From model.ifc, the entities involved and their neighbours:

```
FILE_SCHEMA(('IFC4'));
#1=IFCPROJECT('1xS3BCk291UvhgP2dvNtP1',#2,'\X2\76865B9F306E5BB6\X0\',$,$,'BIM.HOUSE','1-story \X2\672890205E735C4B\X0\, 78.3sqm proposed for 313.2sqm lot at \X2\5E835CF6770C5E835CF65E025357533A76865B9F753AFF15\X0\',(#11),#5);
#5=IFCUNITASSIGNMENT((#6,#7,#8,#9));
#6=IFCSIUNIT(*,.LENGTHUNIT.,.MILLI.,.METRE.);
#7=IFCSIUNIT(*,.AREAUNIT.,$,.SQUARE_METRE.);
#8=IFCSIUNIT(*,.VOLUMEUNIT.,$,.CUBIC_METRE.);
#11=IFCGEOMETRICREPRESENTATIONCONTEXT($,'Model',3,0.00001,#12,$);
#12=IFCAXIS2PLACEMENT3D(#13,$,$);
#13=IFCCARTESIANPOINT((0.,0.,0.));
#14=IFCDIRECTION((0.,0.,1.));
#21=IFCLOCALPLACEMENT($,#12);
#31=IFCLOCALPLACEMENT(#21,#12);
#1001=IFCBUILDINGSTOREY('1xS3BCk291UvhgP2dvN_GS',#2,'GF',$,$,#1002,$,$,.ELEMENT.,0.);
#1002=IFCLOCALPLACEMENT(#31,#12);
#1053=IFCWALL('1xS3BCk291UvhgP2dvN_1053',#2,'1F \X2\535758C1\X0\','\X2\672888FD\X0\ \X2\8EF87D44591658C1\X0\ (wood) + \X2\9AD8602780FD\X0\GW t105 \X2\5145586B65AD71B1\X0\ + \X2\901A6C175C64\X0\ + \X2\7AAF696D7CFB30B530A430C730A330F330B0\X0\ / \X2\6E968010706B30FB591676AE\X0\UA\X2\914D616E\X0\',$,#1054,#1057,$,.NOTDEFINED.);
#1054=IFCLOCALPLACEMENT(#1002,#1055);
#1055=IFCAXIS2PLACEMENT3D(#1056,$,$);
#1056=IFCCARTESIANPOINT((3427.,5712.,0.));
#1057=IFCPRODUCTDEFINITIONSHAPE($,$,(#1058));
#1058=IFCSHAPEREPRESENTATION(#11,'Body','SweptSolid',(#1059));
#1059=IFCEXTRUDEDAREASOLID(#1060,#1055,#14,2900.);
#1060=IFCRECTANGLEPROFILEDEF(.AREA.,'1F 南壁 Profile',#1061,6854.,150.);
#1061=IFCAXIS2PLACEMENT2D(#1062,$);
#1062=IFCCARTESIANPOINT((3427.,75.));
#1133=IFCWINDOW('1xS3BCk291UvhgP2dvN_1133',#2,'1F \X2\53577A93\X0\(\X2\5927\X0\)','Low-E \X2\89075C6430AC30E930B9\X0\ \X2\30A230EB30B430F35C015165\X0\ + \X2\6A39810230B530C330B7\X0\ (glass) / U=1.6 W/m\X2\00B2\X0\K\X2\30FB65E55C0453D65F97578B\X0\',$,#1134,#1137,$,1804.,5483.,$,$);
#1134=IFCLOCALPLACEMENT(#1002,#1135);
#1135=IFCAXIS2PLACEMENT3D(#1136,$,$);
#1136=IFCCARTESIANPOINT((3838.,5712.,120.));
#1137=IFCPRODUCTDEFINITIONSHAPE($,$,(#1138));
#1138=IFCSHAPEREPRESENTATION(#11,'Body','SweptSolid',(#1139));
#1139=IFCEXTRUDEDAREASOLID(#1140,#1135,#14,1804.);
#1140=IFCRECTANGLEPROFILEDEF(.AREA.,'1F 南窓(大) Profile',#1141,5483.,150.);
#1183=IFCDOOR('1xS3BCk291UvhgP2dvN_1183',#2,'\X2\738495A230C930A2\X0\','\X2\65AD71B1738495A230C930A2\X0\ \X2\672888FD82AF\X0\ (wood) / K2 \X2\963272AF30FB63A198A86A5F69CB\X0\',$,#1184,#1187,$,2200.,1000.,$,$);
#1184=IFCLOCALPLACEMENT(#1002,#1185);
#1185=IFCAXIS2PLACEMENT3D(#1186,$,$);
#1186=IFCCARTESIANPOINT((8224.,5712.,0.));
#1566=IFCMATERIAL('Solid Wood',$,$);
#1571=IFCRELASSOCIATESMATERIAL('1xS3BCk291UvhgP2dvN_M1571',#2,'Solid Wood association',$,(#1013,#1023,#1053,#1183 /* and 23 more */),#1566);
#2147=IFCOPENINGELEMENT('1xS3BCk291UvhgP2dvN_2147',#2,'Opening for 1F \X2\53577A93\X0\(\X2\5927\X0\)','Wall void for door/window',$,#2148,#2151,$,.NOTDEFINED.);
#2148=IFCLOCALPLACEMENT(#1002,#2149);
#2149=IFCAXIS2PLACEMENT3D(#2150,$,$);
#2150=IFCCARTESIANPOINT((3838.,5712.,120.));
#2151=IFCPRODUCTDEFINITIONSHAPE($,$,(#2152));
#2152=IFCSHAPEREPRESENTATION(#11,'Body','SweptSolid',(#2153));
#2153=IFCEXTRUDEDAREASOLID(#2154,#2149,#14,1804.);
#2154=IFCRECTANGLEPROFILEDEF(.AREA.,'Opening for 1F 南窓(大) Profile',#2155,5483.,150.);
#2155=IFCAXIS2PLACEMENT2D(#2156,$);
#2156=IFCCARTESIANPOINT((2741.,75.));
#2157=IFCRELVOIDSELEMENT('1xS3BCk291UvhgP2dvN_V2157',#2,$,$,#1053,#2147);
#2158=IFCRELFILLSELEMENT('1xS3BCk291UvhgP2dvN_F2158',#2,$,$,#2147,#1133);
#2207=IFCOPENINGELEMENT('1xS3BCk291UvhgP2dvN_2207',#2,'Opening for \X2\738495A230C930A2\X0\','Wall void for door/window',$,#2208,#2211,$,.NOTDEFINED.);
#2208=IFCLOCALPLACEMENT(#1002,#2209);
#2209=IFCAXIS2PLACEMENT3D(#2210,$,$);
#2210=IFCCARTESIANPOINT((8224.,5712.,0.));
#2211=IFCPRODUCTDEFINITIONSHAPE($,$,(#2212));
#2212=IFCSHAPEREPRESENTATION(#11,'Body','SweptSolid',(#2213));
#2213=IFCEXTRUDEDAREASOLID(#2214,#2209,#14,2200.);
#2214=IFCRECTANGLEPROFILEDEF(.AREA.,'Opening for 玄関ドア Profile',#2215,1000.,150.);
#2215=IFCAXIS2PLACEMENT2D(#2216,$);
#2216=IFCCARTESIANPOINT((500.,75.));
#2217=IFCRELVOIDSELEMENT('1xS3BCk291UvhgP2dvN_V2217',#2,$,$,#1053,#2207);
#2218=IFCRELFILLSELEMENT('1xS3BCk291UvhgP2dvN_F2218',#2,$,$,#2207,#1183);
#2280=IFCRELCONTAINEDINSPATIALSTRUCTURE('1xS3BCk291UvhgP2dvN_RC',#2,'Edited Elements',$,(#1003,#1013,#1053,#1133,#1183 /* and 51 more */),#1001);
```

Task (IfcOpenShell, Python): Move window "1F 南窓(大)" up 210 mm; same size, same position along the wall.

```python
import numpy as np
import ifcopenshell
import ifcopenshell.api.geometry
import ifcopenshell.util.placement
import ifcopenshell.util.unit

model = ifcopenshell.open("model.ifc")
unit_scale = ifcopenshell.util.unit.calculate_unit_scale(model)

window = model.by_guid("1xS3BCk291UvhgP2dvN_1133")
opening = window.FillsVoids[0].RelatingOpeningElement
dz = 0.21 / unit_scale

shift = np.array([0.0, 0.0, dz])
# The window is not placed relative to its opening, so move both.
for product in (opening, window):
    matrix = ifcopenshell.util.placement.get_local_placement(product.ObjectPlacement)
    matrix[:3, 3] += shift
    ifcopenshell.api.geometry.edit_object_placement(model, product=product, matrix=matrix, is_si=False)

print(f"moved by {dz * unit_scale:+.3f} m")

model.write("model_edited.ifc")
```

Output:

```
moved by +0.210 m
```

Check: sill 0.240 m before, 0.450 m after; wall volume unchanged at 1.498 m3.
